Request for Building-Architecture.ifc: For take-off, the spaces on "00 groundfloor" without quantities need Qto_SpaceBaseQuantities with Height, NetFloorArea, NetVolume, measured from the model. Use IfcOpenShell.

First a look at what the model holds.

```python
import ifcopenshell
import ifcopenshell.util.element
import ifcopenshell.util.unit

model = ifcopenshell.open("Building-Architecture.ifc")
print(model.schema)
for unit_type in ("LENGTHUNIT", "AREAUNIT", "VOLUMEUNIT"):
    print(unit_type, ifcopenshell.util.unit.calculate_unit_scale(model, unit_type))
storey = next(s for s in model.by_type("IfcBuildingStorey") if s.Name == "00 groundfloor")
spaces = [e for e in ifcopenshell.util.element.get_decomposition(storey) if e.is_a("IfcSpace")]
for e in sorted(spaces, key=lambda e: e.id()):
    print(e.id(), e.is_a(), e.Name, list(ifcopenshell.util.element.get_psets(e, qtos_only=True)), sep=" | ")
```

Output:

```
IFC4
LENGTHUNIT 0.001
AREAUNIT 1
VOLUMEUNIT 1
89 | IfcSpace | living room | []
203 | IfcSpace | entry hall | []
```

```python
import ifcopenshell
import ifcopenshell.api.pset
import ifcopenshell.geom
import ifcopenshell.util.element
import ifcopenshell.util.shape
import ifcopenshell.util.unit

model = ifcopenshell.open("Building-Architecture.ifc")
unit_scale = ifcopenshell.util.unit.calculate_unit_scale(model)
area_scale = ifcopenshell.util.unit.calculate_unit_scale(model, "AREAUNIT")
volume_scale = ifcopenshell.util.unit.calculate_unit_scale(model, "VOLUMEUNIT")
settings = ifcopenshell.geom.settings()

storey = next(s for s in model.by_type("IfcBuildingStorey") if s.Name == "00 groundfloor")
spaces = [e for e in ifcopenshell.util.element.get_decomposition(storey) if e.is_a("IfcSpace")]

for e in sorted(spaces, key=lambda e: e.id()):
    if ifcopenshell.util.element.get_psets(e, qtos_only=True, should_inherit=False):
        continue
    # Geometry comes back in metres, in the element's own axes.
    shape = ifcopenshell.geom.create_shape(settings, e)
    values = {
        "Height": ifcopenshell.util.shape.get_z(shape.geometry) / unit_scale,
        "NetFloorArea": ifcopenshell.util.shape.get_footprint_area(shape.geometry) / area_scale,
        "NetVolume": ifcopenshell.util.shape.get_volume(shape.geometry) / volume_scale,
    }
    qto = ifcopenshell.api.pset.add_qto(model, product=e, name="Qto_SpaceBaseQuantities")
    ifcopenshell.api.pset.edit_qto(model, qto=qto, properties=values)
    print(e.id(), {k: round(v, 3) for k, v in values.items()})

model.write("Building-Architecture_updated.ifc")
```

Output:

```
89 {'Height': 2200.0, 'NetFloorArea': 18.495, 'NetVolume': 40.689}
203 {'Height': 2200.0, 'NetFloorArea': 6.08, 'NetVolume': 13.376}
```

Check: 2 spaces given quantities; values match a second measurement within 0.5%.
